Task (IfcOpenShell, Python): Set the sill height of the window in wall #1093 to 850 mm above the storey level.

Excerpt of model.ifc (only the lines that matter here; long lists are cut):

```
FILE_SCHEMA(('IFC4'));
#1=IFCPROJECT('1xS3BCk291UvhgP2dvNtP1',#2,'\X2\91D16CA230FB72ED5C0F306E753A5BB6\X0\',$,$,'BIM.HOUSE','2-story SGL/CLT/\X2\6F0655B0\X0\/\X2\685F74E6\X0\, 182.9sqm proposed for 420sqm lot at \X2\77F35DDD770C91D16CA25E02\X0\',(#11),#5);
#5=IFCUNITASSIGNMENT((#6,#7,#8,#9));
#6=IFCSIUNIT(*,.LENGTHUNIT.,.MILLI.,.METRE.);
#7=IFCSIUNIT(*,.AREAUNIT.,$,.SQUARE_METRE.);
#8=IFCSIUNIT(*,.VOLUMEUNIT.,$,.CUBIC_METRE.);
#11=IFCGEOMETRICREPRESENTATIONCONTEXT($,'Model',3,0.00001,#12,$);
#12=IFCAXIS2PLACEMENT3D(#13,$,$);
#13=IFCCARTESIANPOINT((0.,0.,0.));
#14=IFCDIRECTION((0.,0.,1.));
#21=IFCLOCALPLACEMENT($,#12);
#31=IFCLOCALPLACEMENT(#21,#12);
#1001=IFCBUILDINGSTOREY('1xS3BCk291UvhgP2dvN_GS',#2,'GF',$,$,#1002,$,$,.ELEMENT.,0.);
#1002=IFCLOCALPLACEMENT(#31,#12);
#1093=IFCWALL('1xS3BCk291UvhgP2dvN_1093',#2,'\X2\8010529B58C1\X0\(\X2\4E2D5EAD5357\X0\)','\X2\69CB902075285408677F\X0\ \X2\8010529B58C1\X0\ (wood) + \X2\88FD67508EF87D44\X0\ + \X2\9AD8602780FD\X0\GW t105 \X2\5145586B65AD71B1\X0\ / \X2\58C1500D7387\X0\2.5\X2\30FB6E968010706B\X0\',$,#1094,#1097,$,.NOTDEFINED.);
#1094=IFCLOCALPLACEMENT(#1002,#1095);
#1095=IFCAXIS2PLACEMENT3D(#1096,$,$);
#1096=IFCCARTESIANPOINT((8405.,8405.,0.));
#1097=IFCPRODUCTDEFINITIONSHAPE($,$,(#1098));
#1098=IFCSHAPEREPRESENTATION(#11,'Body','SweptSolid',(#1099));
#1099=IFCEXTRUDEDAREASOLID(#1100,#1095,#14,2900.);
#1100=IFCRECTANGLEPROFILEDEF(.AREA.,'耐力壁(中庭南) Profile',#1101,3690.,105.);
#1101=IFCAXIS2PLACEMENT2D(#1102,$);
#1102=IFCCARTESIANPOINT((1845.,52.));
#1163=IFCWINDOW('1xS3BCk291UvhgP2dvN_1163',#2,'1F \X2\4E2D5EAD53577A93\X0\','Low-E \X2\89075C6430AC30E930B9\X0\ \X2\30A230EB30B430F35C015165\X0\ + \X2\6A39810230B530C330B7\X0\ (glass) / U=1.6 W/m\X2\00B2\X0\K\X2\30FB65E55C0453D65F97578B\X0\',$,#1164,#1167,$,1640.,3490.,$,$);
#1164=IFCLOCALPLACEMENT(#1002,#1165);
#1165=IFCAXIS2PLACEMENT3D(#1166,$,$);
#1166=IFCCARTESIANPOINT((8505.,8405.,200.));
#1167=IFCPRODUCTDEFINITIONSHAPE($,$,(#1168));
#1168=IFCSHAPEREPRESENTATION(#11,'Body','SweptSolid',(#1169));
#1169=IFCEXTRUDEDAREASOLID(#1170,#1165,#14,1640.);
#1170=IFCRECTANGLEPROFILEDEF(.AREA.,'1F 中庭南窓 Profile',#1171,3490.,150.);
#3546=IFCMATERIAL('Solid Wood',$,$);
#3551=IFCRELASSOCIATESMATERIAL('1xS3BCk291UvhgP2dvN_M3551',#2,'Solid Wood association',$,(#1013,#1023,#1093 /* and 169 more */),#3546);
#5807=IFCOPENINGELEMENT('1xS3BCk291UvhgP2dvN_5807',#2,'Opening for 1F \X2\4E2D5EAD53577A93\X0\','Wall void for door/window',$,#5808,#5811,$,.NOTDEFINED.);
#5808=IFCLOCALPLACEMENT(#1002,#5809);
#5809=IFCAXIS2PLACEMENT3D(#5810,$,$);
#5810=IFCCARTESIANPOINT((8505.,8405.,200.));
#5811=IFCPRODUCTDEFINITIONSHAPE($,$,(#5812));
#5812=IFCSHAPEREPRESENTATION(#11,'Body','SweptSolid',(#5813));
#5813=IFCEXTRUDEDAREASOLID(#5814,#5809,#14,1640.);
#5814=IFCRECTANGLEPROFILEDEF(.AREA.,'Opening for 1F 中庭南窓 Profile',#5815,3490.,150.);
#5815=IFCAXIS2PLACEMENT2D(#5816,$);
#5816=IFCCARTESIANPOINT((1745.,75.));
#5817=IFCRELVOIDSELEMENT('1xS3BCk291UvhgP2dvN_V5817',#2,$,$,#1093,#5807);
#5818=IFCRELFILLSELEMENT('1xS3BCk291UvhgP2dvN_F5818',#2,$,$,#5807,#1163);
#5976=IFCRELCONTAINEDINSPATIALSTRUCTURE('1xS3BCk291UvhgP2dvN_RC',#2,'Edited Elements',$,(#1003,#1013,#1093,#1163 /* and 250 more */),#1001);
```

```python
import numpy as np
import ifcopenshell
import ifcopenshell.api.geometry
import ifcopenshell.geom
import ifcopenshell.util.element
import ifcopenshell.util.placement
import ifcopenshell.util.shape
import ifcopenshell.util.unit

model = ifcopenshell.open("model.ifc")
unit_scale = ifcopenshell.util.unit.calculate_unit_scale(model)

window = model.by_guid("1xS3BCk291UvhgP2dvN_1163")
opening = window.FillsVoids[0].RelatingOpeningElement
storey = ifcopenshell.util.element.get_container(window, ifc_class="IfcBuildingStorey")
level = ifcopenshell.util.placement.get_local_placement(storey.ObjectPlacement)[2, 3]

# The opening's origin need not be at the sill, so measure its lowest point.
shape = ifcopenshell.geom.create_shape(ifcopenshell.geom.settings(), opening)
bottom = ifcopenshell.util.shape.get_shape_bottom_elevation(shape, shape.geometry) / unit_scale
dz = level + 850.0 - bottom

shift = np.array([0.0, 0.0, dz])
# The window is not placed relative to its opening, so move both.
for product in (opening, window):
    matrix = ifcopenshell.util.placement.get_local_placement(product.ObjectPlacement)
    matrix[:3, 3] += shift
    ifcopenshell.api.geometry.edit_object_placement(model, product=product, matrix=matrix, is_si=False)

print(f"moved by {dz * unit_scale:+.3f} m")

model.write("model_v2.ifc")
```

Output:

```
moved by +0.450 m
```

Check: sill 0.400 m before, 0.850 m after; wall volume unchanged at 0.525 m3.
